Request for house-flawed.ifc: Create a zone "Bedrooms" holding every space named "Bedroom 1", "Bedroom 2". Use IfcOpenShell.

First a look at what the model holds.

```python
import ifcopenshell

model = ifcopenshell.open("house-flawed.ifc")
print(model.schema)
seen = {}
for space in model.by_type("IfcSpace"):
    seen[space.LongName] = seen.get(space.LongName, 0) + 1
for name, count in sorted(seen.items(), key=str):
    print(count, "x", name)
print("zones:", [z.Name for z in model.by_type("IfcZone")][:20])
```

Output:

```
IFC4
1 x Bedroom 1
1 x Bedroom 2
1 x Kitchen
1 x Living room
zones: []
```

```python
import ifcopenshell
import ifcopenshell.api.group
import ifcopenshell.api.root

model = ifcopenshell.open("house-flawed.ifc")

names = {"Bedroom 1", "Bedroom 2"}
spaces = [s for s in model.by_type("IfcSpace") if s.LongName in names]

zone = ifcopenshell.api.root.create_entity(model, ifc_class="IfcZone", name="Bedrooms")
ifcopenshell.api.group.assign_group(model, products=spaces, group=zone)
print(len(spaces), "spaces in", zone.Name)

model.write("house-flawed_rev.ifc")
```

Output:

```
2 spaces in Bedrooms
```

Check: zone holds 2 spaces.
